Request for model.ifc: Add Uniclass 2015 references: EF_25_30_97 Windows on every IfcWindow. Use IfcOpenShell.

First a look at what the model holds.

```python
import ifcopenshell

model = ifcopenshell.open("model.ifc")
print(model.schema)
print("classifications:", [c.Name for c in model.by_type("IfcClassification")])
for ifc_class in ("IfcDoor", "IfcRoof", "IfcStair", "IfcWall", "IfcWindow"):
    print(ifc_class, len(model.by_type(ifc_class)))
```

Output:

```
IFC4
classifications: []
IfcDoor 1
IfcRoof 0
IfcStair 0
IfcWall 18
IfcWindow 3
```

```python
import ifcopenshell
import ifcopenshell.api.classification

model = ifcopenshell.open("model.ifc")

system = ifcopenshell.api.classification.add_classification(model, classification="Uniclass 2015")

codes = {
    "IfcWindow": ("EF_25_30_97", "Windows"),
}
for ifc_class, (code, name) in codes.items():
    products = model.by_type(ifc_class)
    ifcopenshell.api.classification.add_reference(
        model, products=products, classification=system, identification=code, name=name
    )
    print(code, len(products))

model.write("model_v2.ifc")
```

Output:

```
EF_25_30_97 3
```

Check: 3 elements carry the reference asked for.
